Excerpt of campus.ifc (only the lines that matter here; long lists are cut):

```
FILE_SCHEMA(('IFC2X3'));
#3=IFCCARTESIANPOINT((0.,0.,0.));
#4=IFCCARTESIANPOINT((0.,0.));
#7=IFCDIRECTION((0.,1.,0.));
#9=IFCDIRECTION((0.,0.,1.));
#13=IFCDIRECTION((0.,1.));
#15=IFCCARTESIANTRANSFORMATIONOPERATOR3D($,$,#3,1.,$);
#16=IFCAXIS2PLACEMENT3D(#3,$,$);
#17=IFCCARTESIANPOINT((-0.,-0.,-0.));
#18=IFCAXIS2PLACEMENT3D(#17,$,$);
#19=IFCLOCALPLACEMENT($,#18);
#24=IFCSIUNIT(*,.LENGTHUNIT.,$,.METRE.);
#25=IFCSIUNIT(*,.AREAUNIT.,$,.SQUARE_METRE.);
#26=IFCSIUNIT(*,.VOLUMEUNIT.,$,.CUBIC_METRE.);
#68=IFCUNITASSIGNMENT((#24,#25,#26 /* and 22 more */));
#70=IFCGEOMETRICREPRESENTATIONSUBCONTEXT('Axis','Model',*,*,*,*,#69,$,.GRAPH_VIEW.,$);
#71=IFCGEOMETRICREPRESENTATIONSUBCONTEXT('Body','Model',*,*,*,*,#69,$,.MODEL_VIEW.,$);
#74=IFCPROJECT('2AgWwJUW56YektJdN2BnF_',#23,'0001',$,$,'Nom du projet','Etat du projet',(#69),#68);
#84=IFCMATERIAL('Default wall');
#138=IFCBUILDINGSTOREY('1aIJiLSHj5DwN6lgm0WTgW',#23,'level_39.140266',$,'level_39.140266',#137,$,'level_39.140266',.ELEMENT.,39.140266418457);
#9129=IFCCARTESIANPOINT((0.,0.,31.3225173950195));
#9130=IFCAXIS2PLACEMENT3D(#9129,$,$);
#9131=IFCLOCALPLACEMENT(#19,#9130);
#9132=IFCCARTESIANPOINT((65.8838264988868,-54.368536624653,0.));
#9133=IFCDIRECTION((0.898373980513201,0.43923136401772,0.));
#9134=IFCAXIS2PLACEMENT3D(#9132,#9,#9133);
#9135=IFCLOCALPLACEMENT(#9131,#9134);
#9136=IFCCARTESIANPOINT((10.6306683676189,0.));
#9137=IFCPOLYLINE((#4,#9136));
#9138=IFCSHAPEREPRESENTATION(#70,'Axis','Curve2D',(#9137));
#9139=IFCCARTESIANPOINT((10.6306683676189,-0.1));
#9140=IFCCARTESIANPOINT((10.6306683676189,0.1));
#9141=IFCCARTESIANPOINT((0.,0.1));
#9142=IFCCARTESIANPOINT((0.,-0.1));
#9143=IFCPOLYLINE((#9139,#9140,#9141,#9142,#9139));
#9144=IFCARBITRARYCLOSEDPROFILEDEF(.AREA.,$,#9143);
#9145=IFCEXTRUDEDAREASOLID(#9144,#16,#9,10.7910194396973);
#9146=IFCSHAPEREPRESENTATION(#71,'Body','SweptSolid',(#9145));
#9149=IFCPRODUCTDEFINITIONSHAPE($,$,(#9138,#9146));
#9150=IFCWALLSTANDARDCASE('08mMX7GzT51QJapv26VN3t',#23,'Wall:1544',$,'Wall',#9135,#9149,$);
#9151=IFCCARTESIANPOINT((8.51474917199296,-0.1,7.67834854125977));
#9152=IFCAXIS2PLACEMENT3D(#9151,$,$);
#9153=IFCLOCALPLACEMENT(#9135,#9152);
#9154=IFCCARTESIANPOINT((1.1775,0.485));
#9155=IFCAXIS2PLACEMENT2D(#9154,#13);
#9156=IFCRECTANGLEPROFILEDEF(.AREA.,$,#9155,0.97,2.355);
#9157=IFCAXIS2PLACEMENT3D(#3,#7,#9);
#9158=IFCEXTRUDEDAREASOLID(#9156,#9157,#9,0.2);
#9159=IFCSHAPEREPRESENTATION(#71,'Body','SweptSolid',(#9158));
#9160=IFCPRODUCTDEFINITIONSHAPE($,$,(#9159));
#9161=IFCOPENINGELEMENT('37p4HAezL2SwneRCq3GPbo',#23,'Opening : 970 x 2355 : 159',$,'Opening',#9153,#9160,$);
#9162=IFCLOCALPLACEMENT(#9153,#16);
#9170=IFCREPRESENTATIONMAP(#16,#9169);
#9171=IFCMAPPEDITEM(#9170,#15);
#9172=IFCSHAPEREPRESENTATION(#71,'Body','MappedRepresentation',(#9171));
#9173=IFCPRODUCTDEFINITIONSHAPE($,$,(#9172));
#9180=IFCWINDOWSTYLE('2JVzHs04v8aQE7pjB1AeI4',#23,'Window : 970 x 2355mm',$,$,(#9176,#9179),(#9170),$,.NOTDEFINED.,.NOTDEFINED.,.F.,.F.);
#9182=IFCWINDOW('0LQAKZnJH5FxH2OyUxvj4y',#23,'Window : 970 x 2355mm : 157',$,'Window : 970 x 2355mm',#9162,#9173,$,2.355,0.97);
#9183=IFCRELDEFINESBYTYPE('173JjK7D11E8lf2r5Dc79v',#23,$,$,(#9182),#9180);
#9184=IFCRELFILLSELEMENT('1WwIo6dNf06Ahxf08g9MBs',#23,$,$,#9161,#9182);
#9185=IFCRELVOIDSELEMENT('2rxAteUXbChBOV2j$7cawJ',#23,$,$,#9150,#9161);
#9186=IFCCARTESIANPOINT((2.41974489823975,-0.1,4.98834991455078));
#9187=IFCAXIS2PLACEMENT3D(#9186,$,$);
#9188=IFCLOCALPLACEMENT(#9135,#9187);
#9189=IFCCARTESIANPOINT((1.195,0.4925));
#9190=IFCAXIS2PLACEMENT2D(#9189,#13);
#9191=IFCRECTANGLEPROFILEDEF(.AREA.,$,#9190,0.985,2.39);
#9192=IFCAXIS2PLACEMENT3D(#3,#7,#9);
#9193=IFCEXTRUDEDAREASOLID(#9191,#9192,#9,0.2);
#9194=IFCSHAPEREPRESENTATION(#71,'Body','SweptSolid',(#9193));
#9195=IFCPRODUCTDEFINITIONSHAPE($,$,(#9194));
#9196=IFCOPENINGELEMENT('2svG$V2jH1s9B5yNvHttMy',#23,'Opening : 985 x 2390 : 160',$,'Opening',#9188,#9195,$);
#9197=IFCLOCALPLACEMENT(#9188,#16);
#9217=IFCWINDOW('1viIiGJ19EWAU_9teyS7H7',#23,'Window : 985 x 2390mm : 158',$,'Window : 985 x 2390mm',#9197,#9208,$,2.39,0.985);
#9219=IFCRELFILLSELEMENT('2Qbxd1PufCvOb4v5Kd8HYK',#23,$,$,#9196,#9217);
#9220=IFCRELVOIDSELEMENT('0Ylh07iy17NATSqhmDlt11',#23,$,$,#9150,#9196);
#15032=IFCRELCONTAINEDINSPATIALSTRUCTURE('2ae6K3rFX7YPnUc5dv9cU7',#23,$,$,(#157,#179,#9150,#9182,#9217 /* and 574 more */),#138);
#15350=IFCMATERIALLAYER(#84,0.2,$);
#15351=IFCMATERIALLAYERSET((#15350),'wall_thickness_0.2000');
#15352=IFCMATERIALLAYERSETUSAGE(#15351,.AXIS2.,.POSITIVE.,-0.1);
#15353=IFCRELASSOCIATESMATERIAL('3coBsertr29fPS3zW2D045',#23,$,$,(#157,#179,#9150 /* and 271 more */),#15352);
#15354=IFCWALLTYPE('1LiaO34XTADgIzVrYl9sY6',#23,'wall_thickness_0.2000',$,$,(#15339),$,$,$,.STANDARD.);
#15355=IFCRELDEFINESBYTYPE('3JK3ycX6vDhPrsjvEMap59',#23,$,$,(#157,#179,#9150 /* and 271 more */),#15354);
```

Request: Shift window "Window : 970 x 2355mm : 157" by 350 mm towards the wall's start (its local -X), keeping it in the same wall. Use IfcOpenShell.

```python
import ifcopenshell
import ifcopenshell.api.geometry
import ifcopenshell.util.placement
import ifcopenshell.util.unit

model = ifcopenshell.open("campus.ifc")
unit_scale = ifcopenshell.util.unit.calculate_unit_scale(model)

window = model.by_guid("0LQAKZnJH5FxH2OyUxvj4y")
opening = window.FillsVoids[0].RelatingOpeningElement
wall = opening.VoidsElements[0].RelatingBuildingElement

wall_matrix = ifcopenshell.util.placement.get_local_placement(wall.ObjectPlacement)
shift = wall_matrix[:3, 0] * -0.35 / unit_scale
before = ifcopenshell.util.placement.get_local_placement(window.ObjectPlacement)[:3, 3].copy()

# The window is placed relative to its opening, so it follows when the opening moves.
matrix = ifcopenshell.util.placement.get_local_placement(opening.ObjectPlacement)
matrix[:3, 3] += shift
ifcopenshell.api.geometry.edit_object_placement(
    model, product=opening, matrix=matrix, is_si=False, should_transform_children=True
)

after = ifcopenshell.util.placement.get_local_placement(window.ObjectPlacement)[:3, 3]
print("window moved by", (after - before).round(3) + 0.0)

model.write("campus-out.ifc")
```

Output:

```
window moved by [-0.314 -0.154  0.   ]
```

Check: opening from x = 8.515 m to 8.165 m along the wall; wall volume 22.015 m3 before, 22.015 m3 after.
